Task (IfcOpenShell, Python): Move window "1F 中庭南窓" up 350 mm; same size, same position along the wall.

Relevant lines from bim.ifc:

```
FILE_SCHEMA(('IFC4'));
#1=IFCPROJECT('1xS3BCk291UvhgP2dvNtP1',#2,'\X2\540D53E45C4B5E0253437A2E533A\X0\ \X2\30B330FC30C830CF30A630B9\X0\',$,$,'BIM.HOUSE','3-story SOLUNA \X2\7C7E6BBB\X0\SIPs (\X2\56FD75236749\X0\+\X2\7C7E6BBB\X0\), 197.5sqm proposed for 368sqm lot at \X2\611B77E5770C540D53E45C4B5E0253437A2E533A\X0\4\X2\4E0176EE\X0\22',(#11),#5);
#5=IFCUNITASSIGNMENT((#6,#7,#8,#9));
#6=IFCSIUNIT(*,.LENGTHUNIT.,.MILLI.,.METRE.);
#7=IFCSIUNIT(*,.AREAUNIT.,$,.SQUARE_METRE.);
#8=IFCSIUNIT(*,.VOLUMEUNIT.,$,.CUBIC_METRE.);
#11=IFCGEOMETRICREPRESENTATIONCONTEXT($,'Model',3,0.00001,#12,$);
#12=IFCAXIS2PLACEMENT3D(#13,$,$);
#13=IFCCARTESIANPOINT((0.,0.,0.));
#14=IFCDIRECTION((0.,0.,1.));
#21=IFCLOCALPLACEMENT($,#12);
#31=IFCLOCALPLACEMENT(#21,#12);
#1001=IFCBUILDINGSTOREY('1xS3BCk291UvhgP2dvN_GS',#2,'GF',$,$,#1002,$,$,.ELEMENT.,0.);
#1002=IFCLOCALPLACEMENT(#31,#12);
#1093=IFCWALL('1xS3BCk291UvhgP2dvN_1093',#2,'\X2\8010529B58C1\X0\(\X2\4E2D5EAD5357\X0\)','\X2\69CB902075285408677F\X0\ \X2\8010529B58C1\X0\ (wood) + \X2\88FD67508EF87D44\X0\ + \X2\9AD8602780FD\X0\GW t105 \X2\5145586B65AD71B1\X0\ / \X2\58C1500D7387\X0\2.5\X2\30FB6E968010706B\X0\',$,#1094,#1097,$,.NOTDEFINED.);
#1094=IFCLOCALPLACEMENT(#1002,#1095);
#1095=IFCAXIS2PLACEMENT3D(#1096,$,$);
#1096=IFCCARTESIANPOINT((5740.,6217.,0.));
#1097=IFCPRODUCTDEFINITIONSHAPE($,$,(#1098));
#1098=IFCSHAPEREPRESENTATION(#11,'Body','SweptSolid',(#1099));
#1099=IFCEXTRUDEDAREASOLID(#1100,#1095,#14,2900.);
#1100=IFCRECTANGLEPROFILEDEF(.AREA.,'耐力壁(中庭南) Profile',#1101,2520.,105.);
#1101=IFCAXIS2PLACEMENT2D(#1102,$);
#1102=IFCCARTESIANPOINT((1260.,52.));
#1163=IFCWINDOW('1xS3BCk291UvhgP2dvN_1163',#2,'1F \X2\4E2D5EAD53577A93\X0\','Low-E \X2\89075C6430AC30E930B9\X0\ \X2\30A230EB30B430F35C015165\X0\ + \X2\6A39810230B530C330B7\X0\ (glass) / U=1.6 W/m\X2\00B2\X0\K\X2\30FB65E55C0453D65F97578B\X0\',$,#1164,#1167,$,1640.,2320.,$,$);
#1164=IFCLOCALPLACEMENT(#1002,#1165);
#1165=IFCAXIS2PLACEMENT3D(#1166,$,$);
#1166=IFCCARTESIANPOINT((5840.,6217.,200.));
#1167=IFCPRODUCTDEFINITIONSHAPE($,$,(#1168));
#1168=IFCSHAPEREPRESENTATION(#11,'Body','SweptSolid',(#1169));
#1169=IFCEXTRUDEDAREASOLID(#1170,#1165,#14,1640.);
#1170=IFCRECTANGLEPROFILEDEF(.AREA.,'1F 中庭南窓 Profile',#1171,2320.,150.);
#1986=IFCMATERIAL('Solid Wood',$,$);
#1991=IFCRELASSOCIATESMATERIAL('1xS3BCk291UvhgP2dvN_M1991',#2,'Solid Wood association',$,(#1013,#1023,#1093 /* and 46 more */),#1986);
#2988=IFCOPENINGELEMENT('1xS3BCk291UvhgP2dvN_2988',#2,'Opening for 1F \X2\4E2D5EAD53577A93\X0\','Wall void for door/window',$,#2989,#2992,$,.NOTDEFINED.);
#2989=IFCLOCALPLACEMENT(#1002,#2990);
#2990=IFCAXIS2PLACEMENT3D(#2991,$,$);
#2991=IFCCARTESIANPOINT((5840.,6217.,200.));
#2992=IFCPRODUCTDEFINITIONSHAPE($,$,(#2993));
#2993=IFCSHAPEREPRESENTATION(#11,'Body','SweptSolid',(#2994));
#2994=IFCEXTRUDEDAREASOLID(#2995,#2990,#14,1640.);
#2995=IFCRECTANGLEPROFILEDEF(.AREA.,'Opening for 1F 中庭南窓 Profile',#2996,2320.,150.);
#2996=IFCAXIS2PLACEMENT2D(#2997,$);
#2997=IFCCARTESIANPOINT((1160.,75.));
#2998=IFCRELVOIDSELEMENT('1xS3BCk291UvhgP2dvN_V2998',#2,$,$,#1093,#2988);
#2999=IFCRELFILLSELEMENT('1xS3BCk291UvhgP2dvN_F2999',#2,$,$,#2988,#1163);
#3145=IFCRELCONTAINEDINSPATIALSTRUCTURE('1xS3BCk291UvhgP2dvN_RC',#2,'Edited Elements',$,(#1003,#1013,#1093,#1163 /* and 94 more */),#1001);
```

```python
import numpy as np
import ifcopenshell
import ifcopenshell.api.geometry
import ifcopenshell.util.placement
import ifcopenshell.util.unit

model = ifcopenshell.open("bim.ifc")
unit_scale = ifcopenshell.util.unit.calculate_unit_scale(model)

window = model.by_id(1163)
opening = window.FillsVoids[0].RelatingOpeningElement
dz = 350.0

shift = np.array([0.0, 0.0, dz])
# The window is not placed relative to its opening, so move both.
for product in (opening, window):
    matrix = ifcopenshell.util.placement.get_local_placement(product.ObjectPlacement)
    matrix[:3, 3] += shift
    ifcopenshell.api.geometry.edit_object_placement(model, product=product, matrix=matrix, is_si=False)

print(f"moved by {dz * unit_scale:+.3f} m")

model.write("bim-out.ifc")
```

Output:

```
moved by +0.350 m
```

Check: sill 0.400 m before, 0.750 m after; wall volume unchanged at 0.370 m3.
